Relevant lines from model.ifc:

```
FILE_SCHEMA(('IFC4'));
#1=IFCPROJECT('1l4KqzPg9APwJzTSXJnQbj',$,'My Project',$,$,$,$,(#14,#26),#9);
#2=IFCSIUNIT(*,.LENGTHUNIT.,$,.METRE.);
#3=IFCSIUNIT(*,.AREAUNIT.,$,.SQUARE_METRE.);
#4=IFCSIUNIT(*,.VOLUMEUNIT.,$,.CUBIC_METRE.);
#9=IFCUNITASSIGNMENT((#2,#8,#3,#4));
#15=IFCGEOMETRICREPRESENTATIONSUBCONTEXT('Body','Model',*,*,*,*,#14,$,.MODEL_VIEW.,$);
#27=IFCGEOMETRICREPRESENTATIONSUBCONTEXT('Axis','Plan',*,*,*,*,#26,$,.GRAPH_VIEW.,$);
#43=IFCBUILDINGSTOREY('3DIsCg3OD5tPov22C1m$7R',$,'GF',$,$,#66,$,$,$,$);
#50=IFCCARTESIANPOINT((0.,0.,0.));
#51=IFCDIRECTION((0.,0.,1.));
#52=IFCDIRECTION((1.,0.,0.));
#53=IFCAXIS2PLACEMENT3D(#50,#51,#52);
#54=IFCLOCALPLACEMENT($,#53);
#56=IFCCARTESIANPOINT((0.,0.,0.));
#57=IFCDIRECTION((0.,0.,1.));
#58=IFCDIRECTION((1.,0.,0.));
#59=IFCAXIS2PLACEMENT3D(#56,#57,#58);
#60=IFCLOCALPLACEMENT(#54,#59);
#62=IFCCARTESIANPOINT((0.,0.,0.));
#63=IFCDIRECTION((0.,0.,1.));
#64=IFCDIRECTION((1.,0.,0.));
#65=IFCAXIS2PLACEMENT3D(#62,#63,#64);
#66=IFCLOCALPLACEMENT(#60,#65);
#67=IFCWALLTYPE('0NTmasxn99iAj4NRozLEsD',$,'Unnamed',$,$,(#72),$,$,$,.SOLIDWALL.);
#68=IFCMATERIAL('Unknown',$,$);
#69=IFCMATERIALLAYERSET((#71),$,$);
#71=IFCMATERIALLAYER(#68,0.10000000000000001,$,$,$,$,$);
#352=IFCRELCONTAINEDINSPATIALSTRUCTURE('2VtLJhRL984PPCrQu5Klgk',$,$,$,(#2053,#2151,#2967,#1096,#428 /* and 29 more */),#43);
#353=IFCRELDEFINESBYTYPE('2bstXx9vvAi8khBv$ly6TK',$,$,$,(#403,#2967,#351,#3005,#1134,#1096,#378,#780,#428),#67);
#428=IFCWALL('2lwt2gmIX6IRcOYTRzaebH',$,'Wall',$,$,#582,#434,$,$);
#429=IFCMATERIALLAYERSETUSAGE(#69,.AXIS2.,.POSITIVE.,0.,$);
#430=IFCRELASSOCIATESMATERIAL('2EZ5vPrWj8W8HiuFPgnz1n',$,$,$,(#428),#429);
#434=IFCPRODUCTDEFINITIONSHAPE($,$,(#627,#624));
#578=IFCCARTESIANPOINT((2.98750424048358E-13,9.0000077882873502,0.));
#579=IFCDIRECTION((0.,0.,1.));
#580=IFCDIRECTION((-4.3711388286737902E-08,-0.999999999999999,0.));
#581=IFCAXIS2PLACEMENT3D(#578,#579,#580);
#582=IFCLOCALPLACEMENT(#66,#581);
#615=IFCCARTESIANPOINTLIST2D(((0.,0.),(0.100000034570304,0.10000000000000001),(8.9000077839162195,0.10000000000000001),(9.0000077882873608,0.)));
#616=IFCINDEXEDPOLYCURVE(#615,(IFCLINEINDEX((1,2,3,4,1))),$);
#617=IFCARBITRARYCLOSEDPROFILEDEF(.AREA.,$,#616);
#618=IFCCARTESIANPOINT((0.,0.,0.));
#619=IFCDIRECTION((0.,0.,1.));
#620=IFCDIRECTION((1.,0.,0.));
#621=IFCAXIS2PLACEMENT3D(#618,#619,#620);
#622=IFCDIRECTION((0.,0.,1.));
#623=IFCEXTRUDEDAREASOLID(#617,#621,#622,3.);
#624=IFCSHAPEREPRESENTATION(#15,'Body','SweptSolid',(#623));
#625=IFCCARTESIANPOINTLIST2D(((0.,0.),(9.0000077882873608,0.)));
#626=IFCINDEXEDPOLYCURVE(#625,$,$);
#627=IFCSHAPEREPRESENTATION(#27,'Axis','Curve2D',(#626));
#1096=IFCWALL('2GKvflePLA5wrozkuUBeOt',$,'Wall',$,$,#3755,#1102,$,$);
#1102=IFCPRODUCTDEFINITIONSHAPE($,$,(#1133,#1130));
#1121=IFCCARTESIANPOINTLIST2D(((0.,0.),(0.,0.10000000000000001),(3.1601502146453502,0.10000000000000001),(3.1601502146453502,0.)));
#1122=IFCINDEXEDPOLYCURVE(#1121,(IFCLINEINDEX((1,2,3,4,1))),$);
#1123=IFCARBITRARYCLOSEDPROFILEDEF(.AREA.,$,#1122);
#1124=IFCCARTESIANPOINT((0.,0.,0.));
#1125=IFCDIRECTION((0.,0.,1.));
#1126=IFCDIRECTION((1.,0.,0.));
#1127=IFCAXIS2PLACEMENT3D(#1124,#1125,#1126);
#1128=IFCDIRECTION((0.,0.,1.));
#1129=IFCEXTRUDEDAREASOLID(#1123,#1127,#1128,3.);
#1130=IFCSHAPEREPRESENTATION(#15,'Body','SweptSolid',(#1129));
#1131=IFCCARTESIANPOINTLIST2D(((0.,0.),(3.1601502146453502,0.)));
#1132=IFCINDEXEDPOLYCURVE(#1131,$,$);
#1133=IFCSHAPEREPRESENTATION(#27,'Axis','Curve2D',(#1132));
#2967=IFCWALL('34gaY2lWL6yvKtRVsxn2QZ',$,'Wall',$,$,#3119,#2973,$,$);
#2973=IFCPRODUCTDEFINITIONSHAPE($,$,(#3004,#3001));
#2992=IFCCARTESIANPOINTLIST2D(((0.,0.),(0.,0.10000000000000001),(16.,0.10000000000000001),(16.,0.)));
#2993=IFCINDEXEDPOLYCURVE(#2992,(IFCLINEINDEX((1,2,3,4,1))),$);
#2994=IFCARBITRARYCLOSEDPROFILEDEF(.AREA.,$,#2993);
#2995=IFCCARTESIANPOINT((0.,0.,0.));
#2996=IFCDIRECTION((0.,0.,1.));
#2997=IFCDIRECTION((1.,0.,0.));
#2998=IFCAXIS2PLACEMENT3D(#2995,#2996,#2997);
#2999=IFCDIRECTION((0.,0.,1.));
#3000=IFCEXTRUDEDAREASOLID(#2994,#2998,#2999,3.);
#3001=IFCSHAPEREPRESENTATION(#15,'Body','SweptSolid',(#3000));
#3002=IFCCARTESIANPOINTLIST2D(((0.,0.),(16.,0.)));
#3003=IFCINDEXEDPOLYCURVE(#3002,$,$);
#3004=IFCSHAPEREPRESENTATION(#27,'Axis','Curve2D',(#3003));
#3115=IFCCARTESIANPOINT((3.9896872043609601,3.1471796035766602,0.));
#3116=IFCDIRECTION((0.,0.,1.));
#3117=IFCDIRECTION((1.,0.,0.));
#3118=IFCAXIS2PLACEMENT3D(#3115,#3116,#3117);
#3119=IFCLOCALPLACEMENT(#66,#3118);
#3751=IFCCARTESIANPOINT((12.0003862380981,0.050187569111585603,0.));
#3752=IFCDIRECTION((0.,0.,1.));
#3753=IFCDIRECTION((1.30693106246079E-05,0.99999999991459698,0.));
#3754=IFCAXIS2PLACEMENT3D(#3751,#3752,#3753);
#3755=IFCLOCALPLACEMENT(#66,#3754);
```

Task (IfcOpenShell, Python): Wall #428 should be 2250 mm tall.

```python
import ifcopenshell
import ifcopenshell.geom
import ifcopenshell.util.representation
import ifcopenshell.util.shape
import ifcopenshell.util.unit

model = ifcopenshell.open("model.ifc")
unit_scale = ifcopenshell.util.unit.calculate_unit_scale(model)
settings = ifcopenshell.geom.settings()


def volume(element):
    """Net volume in cubic metres, openings subtracted."""
    shape = ifcopenshell.geom.create_shape(settings, element)
    return ifcopenshell.util.shape.get_volume(shape.geometry)


wall = model.by_guid("2lwt2gmIX6IRcOYTRzaebH")
before = volume(wall)

body = ifcopenshell.util.representation.get_representation(wall, "Model", "Body")
solid = body.Items[0]
old_height = solid.Depth
solid.Depth = 2.25 / unit_scale
after = volume(wall)

print(f"height {old_height:g} -> {solid.Depth:g}, volume {before:.3f} -> {after:.3f} m3")

model.write("model_updated.ifc")
```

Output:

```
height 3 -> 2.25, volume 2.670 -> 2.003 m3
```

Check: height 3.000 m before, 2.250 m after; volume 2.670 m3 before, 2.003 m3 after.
